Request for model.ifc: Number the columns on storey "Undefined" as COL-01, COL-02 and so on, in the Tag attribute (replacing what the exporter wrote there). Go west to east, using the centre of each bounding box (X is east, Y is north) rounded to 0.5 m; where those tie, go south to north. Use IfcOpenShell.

First a look at what the model holds.

```python
import ifcopenshell
import ifcopenshell.util.element
import ifcopenshell.util.placement

model = ifcopenshell.open("model.ifc")
print(model.schema)
storey = next(s for s in model.by_type("IfcBuildingStorey") if s.Name == "Undefined")
columns = [e for e in ifcopenshell.util.element.get_decomposition(storey) if e.is_a("IfcColumn")]
for e in sorted(columns, key=lambda e: e.id()):
    origin = ifcopenshell.util.placement.get_local_placement(e.ObjectPlacement)[:3, 3]
    print(e.id(), e.Tag, e.Name, origin.round(2) + 0.0, sep=" | ")
```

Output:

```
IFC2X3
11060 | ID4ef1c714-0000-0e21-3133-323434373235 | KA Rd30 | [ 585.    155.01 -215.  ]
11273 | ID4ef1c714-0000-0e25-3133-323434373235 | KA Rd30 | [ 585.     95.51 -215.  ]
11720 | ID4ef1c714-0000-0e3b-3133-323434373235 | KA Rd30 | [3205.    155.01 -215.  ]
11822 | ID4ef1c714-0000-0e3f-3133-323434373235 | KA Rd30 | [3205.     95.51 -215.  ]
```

```python
import ifcopenshell
import ifcopenshell.geom
import ifcopenshell.util.element
import ifcopenshell.util.shape

model = ifcopenshell.open("model.ifc")
settings = ifcopenshell.geom.settings()
settings.set("use-world-coords", True)


def centre(element):
    shape = ifcopenshell.geom.create_shape(settings, element)
    return ifcopenshell.util.shape.get_bbox_centroid(shape.geometry)


storey = next(s for s in model.by_type("IfcBuildingStorey") if s.Name == "Undefined")
columns = [e for e in ifcopenshell.util.element.get_decomposition(storey) if e.is_a("IfcColumn")]

# Insertion points can sit at a corner or the storey origin, so sort by the geometry (in metres).
centres = {e: centre(e) for e in columns}
columns.sort(key=lambda e: (round(centres[e][0] / 0.5), centres[e][1]))

for i, e in enumerate(columns, start=1):
    number = f"COL-{i:02d}"
    e.Tag = number
    print(e.id(), number)

model.write("model_updated.ifc")
```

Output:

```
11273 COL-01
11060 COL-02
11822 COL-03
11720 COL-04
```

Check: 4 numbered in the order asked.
